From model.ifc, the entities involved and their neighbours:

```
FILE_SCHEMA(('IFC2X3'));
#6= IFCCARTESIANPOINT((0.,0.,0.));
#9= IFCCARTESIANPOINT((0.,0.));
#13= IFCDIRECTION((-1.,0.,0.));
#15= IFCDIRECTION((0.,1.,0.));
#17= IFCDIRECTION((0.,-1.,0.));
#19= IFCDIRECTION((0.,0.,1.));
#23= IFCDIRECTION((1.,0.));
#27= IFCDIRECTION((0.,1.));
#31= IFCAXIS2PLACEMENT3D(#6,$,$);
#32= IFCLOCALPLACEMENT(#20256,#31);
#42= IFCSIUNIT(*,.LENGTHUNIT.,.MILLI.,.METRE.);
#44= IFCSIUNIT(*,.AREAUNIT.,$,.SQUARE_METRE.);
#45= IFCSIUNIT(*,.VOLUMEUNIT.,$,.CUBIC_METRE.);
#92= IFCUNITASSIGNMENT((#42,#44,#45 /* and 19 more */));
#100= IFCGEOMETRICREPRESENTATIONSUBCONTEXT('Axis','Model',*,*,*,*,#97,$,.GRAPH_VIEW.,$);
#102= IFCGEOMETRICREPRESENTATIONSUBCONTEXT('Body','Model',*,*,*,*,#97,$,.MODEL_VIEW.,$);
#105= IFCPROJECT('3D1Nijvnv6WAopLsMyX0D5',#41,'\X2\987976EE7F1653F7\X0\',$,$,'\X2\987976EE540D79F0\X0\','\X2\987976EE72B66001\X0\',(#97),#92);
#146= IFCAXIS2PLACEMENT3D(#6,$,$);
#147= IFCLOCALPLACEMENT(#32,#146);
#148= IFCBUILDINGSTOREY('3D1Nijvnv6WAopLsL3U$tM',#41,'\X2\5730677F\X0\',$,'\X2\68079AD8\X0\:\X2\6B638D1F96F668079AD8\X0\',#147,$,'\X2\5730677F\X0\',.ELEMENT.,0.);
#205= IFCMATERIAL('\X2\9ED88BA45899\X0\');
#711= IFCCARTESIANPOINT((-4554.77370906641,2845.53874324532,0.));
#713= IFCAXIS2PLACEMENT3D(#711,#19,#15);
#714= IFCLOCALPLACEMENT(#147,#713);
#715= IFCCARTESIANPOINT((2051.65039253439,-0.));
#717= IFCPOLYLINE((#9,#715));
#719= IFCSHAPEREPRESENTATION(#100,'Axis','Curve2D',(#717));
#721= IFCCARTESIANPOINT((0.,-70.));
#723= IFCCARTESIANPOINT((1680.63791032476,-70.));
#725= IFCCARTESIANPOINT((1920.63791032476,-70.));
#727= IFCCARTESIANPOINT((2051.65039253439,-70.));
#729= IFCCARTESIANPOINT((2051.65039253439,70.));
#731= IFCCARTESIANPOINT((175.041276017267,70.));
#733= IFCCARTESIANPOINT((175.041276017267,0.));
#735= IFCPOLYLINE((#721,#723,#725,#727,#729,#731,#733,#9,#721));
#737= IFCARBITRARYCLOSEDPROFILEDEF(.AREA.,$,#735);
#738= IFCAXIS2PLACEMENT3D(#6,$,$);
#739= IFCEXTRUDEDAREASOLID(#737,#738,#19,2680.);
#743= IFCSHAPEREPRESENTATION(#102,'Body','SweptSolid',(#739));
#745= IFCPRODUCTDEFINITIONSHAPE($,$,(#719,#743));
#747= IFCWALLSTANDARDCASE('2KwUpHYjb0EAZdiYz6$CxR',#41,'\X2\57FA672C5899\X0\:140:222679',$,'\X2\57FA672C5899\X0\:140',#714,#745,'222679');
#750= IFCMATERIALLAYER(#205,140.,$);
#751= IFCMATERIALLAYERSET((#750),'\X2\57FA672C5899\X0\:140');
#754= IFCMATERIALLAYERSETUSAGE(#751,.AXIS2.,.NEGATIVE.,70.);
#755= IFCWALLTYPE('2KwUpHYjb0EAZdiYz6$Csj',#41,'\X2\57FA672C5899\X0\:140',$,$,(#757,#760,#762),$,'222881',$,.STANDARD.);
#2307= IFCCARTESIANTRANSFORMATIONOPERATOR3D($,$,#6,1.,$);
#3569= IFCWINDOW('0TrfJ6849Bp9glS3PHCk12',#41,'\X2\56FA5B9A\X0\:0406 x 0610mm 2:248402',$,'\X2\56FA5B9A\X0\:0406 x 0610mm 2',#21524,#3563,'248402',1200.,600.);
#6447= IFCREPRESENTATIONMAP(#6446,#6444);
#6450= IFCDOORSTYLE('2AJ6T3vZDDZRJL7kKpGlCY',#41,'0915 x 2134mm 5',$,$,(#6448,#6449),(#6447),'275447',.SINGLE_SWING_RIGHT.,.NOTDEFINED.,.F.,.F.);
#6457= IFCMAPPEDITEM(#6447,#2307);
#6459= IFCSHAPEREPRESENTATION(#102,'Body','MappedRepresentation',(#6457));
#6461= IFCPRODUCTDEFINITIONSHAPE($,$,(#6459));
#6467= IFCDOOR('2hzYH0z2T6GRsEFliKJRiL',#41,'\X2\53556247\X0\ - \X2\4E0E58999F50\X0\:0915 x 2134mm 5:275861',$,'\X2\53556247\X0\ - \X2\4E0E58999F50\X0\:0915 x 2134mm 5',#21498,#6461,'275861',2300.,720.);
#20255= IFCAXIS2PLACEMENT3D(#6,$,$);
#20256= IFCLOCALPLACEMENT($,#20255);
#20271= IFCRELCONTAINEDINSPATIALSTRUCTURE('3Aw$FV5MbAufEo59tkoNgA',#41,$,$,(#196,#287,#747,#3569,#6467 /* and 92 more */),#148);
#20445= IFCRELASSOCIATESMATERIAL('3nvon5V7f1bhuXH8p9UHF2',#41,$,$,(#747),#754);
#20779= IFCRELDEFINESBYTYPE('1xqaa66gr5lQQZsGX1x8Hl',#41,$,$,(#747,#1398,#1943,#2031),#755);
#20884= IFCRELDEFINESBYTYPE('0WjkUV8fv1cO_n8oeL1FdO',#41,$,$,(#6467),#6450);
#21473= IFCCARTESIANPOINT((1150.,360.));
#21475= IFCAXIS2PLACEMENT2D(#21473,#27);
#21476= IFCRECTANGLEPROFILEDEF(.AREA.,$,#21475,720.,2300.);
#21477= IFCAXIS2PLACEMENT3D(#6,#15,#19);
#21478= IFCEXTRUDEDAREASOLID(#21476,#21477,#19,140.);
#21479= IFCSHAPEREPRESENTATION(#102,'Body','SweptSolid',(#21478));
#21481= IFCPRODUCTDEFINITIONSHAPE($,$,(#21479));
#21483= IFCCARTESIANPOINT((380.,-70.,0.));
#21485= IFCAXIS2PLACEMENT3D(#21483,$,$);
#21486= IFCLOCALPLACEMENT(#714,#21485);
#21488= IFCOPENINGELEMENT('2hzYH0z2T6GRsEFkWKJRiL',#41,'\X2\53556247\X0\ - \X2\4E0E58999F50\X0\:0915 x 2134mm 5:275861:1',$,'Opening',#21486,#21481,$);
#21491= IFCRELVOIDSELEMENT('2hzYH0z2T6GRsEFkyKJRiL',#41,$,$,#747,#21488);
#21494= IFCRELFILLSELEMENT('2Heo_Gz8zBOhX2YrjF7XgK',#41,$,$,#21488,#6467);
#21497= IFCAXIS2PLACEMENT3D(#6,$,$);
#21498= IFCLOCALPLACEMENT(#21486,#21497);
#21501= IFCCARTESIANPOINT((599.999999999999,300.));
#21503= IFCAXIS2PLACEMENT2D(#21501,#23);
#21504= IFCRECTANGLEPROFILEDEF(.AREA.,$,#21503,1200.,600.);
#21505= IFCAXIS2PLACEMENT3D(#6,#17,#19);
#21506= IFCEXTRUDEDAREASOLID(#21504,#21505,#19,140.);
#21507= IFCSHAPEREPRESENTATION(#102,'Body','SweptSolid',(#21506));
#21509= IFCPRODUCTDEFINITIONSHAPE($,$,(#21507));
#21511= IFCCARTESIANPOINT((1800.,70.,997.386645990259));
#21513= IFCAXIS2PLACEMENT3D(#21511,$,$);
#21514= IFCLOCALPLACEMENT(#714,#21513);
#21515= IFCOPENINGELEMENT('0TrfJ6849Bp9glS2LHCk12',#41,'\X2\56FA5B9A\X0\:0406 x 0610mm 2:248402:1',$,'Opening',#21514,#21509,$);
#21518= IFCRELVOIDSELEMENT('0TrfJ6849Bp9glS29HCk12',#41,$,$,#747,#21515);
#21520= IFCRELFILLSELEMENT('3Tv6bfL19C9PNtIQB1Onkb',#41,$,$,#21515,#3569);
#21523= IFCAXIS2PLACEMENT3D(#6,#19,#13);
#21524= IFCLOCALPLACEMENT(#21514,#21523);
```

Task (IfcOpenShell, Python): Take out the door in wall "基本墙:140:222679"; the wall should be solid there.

```python
import ifcopenshell
import ifcopenshell.api.feature
import ifcopenshell.api.root
import ifcopenshell.geom
import ifcopenshell.util.shape

model = ifcopenshell.open("model.ifc")
settings = ifcopenshell.geom.settings()


def volume(element):
    """Net volume in cubic metres, openings subtracted."""
    shape = ifcopenshell.geom.create_shape(settings, element)
    return ifcopenshell.util.shape.get_volume(shape.geometry)


door = model.by_guid("2hzYH0z2T6GRsEFliKJRiL")
opening = door.FillsVoids[0].RelatingOpeningElement
wall = opening.VoidsElements[0].RelatingBuildingElement
before = volume(wall)

ifcopenshell.api.root.remove_product(model, product=door)
ifcopenshell.api.feature.remove_feature(model, feature=opening)

after = volume(wall)

print(f"wall volume {before:.3f} -> {after:.3f} m3")

model.write("model_updated.ifc")
```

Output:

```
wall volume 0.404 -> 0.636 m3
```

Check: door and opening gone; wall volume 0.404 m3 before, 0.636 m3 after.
